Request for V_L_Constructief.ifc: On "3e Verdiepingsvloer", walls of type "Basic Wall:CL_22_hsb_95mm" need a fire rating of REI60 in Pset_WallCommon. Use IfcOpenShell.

First a look at what the model holds.

```python
import ifcopenshell
import ifcopenshell.util.element

model = ifcopenshell.open("V_L_Constructief.ifc")
print(model.schema)
storey = next(s for s in model.by_type("IfcBuildingStorey") if s.Name == "3e Verdiepingsvloer")
walls = [e for e in ifcopenshell.util.element.get_decomposition(storey) if e.is_a("IfcWall")]
seen = {}
for e in walls:
    element_type = ifcopenshell.util.element.get_type(e)
    key = (element_type.Name if element_type != e and element_type else None, ifcopenshell.util.element.get_pset(e, "Pset_WallCommon", "FireRating"))
    seen[key] = seen.get(key, 0) + 1
for (name, value), count in sorted(seen.items(), key=str):
    print(count, "x", name, "|", value)
```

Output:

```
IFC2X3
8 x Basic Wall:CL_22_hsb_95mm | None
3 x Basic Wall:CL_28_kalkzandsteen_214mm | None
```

```python
import ifcopenshell
import ifcopenshell.api.pset
import ifcopenshell.util.element

model = ifcopenshell.open("V_L_Constructief.ifc")

storey = next(s for s in model.by_type("IfcBuildingStorey") if s.Name == "3e Verdiepingsvloer")
walls = [e for e in ifcopenshell.util.element.get_decomposition(storey) if e.is_a("IfcWall")]

count = 0
for e in walls:
    element_type = ifcopenshell.util.element.get_type(e)
    if element_type in (None, e) or element_type.Name != "Basic Wall:CL_22_hsb_95mm":
        continue
    found = ifcopenshell.util.element.get_pset(e, "Pset_WallCommon", should_inherit=False)
    if found:
        pset = model.by_id(found["id"])
        if len(ifcopenshell.util.element.get_elements_by_pset(pset)) > 1:
            pset = ifcopenshell.api.pset.unshare_pset(model, products=[e], pset=pset)[0]
    else:
        pset = ifcopenshell.api.pset.add_pset(model, product=e, name="Pset_WallCommon")
    ifcopenshell.api.pset.edit_pset(model, pset=pset, properties={"FireRating": "REI60"})
    count += 1

print(count, "walls updated")

model.write("V_L_Constructief_rev.ifc")
```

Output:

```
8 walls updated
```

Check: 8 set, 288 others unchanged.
